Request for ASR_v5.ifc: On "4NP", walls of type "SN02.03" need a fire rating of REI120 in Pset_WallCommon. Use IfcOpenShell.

First a look at what the model holds.

```python
import ifcopenshell
import ifcopenshell.util.element

model = ifcopenshell.open("ASR_v5.ifc")
print(model.schema)
storey = next(s for s in model.by_type("IfcBuildingStorey") if s.Name == "4NP")
walls = [e for e in ifcopenshell.util.element.get_decomposition(storey) if e.is_a("IfcWall")]
seen = {}
for e in walls:
    element_type = ifcopenshell.util.element.get_type(e)
    key = (element_type.Name if element_type != e and element_type else None, ifcopenshell.util.element.get_pset(e, "Pset_WallCommon", "FireRating"))
    seen[key] = seen.get(key, 0) + 1
for (name, value), count in sorted(seen.items(), key=str):
    print(count, "x", name, "|", value)
```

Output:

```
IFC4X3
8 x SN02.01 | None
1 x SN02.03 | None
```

```python
import ifcopenshell
import ifcopenshell.api.pset
import ifcopenshell.util.element

model = ifcopenshell.open("ASR_v5.ifc")

storey = next(s for s in model.by_type("IfcBuildingStorey") if s.Name == "4NP")
walls = [e for e in ifcopenshell.util.element.get_decomposition(storey) if e.is_a("IfcWall")]

count = 0
for e in walls:
    element_type = ifcopenshell.util.element.get_type(e)
    if element_type in (None, e) or element_type.Name != "SN02.03":
        continue
    # add_pset returns the element's existing set when there is one.
    pset = ifcopenshell.api.pset.add_pset(model, product=e, name="Pset_WallCommon")
    ifcopenshell.api.pset.edit_pset(model, pset=pset, properties={"FireRating": "REI120"})
    count += 1

print(count, "walls updated")

model.write("ASR_v5-out.ifc")
```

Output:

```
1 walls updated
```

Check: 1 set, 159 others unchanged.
